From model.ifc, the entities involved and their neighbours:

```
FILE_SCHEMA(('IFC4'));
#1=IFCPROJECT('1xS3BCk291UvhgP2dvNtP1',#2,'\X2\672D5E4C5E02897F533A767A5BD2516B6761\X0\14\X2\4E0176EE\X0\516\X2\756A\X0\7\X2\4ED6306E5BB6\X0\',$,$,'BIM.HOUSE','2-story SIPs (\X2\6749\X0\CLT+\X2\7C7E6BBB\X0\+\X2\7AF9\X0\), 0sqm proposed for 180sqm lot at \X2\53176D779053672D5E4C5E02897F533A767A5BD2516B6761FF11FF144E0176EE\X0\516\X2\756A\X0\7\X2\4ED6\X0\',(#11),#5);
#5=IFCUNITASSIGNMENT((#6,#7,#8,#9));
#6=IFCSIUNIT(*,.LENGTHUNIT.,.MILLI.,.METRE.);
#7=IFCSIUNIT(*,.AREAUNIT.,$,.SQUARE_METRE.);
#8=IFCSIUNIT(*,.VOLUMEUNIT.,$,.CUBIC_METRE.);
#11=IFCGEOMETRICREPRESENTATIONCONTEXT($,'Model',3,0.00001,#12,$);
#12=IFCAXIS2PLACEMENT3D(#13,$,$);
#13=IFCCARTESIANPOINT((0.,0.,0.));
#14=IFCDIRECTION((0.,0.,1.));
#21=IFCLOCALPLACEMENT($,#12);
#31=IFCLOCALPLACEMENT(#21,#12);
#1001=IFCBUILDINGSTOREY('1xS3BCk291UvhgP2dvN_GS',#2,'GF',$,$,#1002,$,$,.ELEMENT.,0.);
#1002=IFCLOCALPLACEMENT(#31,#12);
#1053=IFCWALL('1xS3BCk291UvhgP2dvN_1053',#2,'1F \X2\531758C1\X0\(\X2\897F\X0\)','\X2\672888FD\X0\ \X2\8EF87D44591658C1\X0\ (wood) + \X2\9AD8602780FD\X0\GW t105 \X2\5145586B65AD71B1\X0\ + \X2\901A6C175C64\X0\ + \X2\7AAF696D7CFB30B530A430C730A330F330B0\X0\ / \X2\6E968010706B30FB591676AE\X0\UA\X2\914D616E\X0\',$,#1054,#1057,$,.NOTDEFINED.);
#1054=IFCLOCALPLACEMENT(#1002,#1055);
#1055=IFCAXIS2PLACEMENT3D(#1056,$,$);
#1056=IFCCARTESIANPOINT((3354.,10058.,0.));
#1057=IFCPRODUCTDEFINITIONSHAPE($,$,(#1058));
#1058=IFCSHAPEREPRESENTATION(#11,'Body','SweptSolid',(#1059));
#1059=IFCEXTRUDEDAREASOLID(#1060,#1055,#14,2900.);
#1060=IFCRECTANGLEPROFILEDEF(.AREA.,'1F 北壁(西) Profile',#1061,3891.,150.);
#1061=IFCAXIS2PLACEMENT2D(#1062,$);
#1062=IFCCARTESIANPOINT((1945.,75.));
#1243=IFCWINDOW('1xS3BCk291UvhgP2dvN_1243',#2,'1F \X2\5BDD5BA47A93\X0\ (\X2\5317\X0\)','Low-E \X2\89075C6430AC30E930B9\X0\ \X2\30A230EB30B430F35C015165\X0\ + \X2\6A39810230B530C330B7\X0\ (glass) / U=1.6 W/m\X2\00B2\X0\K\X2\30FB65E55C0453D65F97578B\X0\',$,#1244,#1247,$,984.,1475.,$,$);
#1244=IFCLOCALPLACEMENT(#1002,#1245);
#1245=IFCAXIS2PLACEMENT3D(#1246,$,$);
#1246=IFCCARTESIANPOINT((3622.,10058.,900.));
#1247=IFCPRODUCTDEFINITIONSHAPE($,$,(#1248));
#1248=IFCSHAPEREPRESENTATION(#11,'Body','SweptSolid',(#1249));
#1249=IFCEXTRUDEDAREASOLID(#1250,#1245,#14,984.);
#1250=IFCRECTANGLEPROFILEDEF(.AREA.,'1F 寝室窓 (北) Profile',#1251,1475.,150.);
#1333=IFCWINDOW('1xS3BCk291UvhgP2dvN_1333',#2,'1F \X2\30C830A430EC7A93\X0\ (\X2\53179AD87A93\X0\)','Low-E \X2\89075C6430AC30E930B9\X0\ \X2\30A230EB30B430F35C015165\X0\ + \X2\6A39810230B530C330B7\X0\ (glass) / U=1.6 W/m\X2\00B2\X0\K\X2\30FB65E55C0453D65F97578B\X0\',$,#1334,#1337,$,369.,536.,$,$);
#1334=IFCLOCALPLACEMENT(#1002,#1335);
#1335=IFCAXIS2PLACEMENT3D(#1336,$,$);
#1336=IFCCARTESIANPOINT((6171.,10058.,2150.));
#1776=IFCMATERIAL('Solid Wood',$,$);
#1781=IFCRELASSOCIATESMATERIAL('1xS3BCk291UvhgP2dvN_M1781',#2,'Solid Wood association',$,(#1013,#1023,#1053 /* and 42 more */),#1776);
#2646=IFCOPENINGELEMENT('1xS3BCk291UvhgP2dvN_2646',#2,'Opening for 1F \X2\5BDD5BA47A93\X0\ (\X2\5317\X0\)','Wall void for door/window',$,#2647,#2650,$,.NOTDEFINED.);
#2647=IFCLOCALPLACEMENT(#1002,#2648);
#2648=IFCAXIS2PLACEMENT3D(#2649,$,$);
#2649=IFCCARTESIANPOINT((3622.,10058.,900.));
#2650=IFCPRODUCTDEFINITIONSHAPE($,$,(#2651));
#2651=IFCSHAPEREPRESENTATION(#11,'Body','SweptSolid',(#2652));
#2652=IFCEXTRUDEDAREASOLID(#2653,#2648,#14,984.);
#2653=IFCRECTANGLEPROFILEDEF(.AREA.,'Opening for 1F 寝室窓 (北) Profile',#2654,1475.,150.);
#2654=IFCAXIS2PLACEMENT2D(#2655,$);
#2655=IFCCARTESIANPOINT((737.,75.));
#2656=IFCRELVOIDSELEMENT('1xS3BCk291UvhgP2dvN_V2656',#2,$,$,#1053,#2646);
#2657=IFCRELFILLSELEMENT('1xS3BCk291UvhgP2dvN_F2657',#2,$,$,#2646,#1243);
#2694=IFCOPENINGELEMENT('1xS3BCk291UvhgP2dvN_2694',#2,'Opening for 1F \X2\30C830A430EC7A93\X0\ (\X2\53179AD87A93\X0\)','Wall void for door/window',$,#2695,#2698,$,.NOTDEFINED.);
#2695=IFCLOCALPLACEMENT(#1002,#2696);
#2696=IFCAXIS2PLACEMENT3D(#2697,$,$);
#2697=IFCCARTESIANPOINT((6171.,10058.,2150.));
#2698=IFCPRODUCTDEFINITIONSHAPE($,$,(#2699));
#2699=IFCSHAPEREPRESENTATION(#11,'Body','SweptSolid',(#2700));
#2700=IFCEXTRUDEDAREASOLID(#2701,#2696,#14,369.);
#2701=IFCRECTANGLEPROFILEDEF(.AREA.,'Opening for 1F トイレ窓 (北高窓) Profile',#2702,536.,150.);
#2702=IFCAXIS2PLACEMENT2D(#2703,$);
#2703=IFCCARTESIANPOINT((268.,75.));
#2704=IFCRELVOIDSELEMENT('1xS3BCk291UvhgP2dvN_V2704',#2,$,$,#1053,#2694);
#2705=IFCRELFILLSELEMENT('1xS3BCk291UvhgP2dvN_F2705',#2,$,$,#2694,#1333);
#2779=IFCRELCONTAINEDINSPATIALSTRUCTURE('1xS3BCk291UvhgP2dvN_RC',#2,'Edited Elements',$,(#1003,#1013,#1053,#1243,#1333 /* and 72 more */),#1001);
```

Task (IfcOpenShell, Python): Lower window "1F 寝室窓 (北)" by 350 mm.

```python
import numpy as np
import ifcopenshell
import ifcopenshell.api.geometry
import ifcopenshell.util.placement
import ifcopenshell.util.unit

model = ifcopenshell.open("model.ifc")
unit_scale = ifcopenshell.util.unit.calculate_unit_scale(model)

window = model.by_id(1243)
opening = window.FillsVoids[0].RelatingOpeningElement
dz = -350.0

shift = np.array([0.0, 0.0, dz])
# The window is not placed relative to its opening, so move both.
for product in (opening, window):
    matrix = ifcopenshell.util.placement.get_local_placement(product.ObjectPlacement)
    matrix[:3, 3] += shift
    ifcopenshell.api.geometry.edit_object_placement(model, product=product, matrix=matrix, is_si=False)

print(f"moved by {dz * unit_scale:+.3f} m")

model.write("model_v2.ifc")
```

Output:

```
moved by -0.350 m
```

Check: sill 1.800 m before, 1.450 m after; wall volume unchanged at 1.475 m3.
